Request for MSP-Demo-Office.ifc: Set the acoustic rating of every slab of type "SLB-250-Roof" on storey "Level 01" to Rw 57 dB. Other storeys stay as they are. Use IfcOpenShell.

First a look at what the model holds.

```python
import ifcopenshell
import ifcopenshell.util.element

model = ifcopenshell.open("MSP-Demo-Office.ifc")
print(model.schema)
storey = next(s for s in model.by_type("IfcBuildingStorey") if s.Name == "Level 01")
slabs = [e for e in ifcopenshell.util.element.get_decomposition(storey) if e.is_a("IfcSlab")]
seen = {}
for e in slabs:
    element_type = ifcopenshell.util.element.get_type(e)
    key = (element_type.Name if element_type != e and element_type else None, ifcopenshell.util.element.get_pset(e, "Pset_SlabCommon", "AcousticRating"))
    seen[key] = seen.get(key, 0) + 1
for (name, value), count in sorted(seen.items(), key=str):
    print(count, "x", name, "|", value)
```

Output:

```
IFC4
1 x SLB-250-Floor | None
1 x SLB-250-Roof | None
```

```python
import ifcopenshell
import ifcopenshell.api.pset
import ifcopenshell.util.element

model = ifcopenshell.open("MSP-Demo-Office.ifc")

storey = next(s for s in model.by_type("IfcBuildingStorey") if s.Name == "Level 01")
slabs = [e for e in ifcopenshell.util.element.get_decomposition(storey) if e.is_a("IfcSlab")]

count = 0
for e in slabs:
    element_type = ifcopenshell.util.element.get_type(e)
    if element_type in (None, e) or element_type.Name != "SLB-250-Roof":
        continue
    # add_pset returns the element's existing set when there is one.
    pset = ifcopenshell.api.pset.add_pset(model, product=e, name="Pset_SlabCommon")
    ifcopenshell.api.pset.edit_pset(model, pset=pset, properties={"AcousticRating": "Rw 57 dB"})
    count += 1

print(count, "slabs updated")

model.write("MSP-Demo-Office_edited.ifc")
```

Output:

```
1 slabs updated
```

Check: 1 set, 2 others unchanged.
